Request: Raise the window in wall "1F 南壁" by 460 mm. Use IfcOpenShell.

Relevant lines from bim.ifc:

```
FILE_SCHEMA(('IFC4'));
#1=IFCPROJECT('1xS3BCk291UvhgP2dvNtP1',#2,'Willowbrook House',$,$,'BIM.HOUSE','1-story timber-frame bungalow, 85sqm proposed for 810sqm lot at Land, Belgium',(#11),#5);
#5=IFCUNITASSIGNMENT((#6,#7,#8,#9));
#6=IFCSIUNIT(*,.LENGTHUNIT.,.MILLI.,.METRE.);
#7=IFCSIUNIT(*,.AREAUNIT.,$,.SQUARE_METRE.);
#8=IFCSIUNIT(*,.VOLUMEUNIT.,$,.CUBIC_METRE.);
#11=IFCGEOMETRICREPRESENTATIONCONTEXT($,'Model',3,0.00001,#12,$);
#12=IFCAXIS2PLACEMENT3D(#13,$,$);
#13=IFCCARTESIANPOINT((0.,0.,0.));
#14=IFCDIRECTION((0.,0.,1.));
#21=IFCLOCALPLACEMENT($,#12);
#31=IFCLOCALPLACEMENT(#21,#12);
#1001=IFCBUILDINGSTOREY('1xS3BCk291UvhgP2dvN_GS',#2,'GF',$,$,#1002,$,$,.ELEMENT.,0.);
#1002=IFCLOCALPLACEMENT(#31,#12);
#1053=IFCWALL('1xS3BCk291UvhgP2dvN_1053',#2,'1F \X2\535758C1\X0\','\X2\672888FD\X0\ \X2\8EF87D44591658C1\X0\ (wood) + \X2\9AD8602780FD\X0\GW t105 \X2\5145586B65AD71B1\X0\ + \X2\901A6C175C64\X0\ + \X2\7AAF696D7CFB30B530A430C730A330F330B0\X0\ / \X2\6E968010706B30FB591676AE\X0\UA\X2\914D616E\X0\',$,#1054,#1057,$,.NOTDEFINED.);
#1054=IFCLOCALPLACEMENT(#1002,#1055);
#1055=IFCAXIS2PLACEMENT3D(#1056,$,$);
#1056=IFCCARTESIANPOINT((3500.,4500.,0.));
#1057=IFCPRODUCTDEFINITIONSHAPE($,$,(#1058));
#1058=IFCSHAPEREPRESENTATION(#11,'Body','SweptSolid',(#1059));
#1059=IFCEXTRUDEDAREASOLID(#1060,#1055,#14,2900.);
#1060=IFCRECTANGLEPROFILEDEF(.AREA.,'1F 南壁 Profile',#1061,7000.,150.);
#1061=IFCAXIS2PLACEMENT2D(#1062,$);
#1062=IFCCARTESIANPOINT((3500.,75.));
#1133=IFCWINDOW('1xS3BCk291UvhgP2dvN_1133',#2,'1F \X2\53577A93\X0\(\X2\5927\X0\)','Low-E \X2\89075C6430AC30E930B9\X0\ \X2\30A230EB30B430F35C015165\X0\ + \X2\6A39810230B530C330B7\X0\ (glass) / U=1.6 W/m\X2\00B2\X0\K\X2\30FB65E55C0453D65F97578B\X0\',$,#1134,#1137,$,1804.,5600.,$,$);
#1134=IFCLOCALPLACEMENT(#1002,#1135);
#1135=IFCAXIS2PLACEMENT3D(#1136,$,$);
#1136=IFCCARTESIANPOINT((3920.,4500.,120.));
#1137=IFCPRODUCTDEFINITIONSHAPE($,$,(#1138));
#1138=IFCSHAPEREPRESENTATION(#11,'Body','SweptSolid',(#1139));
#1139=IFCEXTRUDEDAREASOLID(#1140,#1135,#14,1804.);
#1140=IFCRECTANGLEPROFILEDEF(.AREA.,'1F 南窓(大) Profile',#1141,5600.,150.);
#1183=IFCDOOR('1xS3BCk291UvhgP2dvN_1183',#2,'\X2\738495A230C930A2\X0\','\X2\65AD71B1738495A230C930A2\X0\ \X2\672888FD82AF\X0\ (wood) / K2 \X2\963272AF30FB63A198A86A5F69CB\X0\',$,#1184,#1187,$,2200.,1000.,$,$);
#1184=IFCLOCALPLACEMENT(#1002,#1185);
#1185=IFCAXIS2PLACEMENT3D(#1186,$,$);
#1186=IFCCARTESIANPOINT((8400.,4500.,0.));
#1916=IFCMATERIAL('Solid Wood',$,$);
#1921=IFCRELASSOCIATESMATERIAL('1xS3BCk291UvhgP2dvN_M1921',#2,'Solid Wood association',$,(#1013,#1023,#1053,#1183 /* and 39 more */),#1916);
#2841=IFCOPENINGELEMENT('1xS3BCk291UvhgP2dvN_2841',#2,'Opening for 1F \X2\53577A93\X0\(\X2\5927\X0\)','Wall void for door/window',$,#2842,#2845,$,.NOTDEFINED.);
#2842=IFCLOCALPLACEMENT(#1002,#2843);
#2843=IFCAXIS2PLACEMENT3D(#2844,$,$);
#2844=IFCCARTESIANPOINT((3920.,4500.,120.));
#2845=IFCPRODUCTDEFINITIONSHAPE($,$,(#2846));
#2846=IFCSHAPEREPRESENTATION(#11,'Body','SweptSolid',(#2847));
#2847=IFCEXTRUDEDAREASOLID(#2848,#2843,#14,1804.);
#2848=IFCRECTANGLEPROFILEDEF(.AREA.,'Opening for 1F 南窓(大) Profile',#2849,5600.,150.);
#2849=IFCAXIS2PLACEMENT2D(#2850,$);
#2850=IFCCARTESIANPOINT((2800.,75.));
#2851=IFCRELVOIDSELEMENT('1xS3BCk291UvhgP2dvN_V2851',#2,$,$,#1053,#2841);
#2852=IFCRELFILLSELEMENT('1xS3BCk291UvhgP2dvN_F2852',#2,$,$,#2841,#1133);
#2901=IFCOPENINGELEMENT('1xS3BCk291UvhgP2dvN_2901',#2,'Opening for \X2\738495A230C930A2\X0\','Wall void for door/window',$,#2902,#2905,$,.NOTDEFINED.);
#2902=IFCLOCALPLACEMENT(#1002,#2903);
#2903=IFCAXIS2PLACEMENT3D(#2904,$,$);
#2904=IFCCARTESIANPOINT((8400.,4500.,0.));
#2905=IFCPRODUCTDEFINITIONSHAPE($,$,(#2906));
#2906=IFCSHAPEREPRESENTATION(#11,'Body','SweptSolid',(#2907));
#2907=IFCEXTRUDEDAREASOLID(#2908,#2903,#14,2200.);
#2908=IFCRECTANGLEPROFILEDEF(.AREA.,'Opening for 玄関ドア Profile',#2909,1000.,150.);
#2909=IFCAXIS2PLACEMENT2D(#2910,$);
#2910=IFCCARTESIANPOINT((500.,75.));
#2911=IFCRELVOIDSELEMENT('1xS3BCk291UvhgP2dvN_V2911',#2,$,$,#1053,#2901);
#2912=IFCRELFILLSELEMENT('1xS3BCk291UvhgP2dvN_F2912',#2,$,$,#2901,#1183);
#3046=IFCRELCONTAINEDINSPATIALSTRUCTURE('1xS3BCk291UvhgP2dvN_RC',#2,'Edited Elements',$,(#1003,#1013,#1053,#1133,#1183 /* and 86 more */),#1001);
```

```python
import numpy as np
import ifcopenshell
import ifcopenshell.api.geometry
import ifcopenshell.util.placement
import ifcopenshell.util.unit

model = ifcopenshell.open("bim.ifc")
unit_scale = ifcopenshell.util.unit.calculate_unit_scale(model)

window = model.by_id(1133)
opening = window.FillsVoids[0].RelatingOpeningElement
dz = 460.0

shift = np.array([0.0, 0.0, dz])
# The window is not placed relative to its opening, so move both.
for product in (opening, window):
    matrix = ifcopenshell.util.placement.get_local_placement(product.ObjectPlacement)
    matrix[:3, 3] += shift
    ifcopenshell.api.geometry.edit_object_placement(model, product=product, matrix=matrix, is_si=False)

print(f"moved by {dz * unit_scale:+.3f} m")

model.write("bim_v2.ifc")
```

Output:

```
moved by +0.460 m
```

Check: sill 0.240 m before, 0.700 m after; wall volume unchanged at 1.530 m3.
